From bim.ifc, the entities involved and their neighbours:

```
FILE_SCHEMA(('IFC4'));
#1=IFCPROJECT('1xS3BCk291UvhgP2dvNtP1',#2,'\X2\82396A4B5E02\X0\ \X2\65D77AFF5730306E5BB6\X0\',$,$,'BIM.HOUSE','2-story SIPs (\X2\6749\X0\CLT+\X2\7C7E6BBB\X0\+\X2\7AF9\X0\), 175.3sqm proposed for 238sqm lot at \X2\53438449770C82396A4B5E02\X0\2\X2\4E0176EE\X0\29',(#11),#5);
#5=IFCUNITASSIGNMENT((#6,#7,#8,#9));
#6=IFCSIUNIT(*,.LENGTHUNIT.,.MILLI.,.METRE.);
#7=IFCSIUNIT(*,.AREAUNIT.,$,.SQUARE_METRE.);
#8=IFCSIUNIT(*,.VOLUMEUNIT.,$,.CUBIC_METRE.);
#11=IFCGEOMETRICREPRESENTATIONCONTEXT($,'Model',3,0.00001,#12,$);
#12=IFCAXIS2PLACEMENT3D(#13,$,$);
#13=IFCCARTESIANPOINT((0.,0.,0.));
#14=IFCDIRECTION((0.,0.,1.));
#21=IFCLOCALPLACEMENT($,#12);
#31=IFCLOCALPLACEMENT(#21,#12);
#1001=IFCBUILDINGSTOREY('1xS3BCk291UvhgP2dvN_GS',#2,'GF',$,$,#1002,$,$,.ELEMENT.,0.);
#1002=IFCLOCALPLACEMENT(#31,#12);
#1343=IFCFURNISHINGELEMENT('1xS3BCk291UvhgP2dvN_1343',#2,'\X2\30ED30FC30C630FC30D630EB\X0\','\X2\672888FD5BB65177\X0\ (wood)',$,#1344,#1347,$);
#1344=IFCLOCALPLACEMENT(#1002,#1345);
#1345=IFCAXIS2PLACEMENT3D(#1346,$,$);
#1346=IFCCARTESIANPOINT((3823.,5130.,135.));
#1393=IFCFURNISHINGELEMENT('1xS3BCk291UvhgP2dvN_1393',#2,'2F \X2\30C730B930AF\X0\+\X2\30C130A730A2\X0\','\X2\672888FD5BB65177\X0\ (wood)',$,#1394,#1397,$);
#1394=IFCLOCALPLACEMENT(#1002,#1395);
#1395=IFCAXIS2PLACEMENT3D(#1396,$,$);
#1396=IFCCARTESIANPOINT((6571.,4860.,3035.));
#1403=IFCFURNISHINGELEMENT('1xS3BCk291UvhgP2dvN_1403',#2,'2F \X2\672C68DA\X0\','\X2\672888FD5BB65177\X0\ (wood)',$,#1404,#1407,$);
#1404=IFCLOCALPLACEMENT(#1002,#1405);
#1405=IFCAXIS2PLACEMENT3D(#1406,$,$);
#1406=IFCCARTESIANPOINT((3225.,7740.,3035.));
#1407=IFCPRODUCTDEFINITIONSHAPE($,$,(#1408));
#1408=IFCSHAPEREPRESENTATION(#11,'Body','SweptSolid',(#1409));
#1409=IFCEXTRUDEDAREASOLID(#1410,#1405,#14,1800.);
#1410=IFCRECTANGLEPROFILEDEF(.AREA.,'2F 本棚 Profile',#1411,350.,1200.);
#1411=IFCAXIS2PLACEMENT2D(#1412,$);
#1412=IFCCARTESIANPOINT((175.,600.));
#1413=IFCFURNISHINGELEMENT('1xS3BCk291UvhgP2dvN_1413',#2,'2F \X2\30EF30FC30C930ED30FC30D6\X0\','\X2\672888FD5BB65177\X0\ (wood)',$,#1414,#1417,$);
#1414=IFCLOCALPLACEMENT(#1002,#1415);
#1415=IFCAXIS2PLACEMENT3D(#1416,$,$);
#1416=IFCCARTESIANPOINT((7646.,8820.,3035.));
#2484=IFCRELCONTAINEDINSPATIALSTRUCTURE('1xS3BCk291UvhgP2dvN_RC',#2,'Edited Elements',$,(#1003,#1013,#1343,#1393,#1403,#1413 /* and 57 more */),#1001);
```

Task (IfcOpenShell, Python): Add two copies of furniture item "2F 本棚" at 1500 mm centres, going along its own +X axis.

```python
import ifcopenshell
import ifcopenshell.api.geometry
import ifcopenshell.api.root
import ifcopenshell.util.element
import ifcopenshell.util.placement

model = ifcopenshell.open("bim.ifc")


def reuse_history(source, copy):
    """copy_class also copies each property set's owner history, people and application; keep the originals."""
    for rel in copy.IsDefinedBy:
        if rel.is_a("IfcRelDefinesByProperties") and (history := rel.RelatingPropertyDefinition.OwnerHistory):
            rel.RelatingPropertyDefinition.OwnerHistory = source.OwnerHistory
            ifcopenshell.util.element.remove_deep2(model, history)


source = model.by_id(1403)
base = ifcopenshell.util.placement.get_local_placement(source.ObjectPlacement)
step = base[:3, 0] * 1500.0

for i in range(1, 3):
    copy = ifcopenshell.api.root.copy_class(model, product=source)
    copy.Representation = ifcopenshell.util.element.copy_deep(
        model, source.Representation, exclude=["IfcGeometricRepresentationContext", "IfcRepresentationMap"]
    )
    reuse_history(source, copy)
    matrix = base.copy()
    matrix[:3, 3] += i * step
    print("added at", matrix[:3, 3].round(3) + 0.0)
    ifcopenshell.api.geometry.edit_object_placement(model, product=copy, matrix=matrix, is_si=False)

model.write("bim_rev.ifc")
```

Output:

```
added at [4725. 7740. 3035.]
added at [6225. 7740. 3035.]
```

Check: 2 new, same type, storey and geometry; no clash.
